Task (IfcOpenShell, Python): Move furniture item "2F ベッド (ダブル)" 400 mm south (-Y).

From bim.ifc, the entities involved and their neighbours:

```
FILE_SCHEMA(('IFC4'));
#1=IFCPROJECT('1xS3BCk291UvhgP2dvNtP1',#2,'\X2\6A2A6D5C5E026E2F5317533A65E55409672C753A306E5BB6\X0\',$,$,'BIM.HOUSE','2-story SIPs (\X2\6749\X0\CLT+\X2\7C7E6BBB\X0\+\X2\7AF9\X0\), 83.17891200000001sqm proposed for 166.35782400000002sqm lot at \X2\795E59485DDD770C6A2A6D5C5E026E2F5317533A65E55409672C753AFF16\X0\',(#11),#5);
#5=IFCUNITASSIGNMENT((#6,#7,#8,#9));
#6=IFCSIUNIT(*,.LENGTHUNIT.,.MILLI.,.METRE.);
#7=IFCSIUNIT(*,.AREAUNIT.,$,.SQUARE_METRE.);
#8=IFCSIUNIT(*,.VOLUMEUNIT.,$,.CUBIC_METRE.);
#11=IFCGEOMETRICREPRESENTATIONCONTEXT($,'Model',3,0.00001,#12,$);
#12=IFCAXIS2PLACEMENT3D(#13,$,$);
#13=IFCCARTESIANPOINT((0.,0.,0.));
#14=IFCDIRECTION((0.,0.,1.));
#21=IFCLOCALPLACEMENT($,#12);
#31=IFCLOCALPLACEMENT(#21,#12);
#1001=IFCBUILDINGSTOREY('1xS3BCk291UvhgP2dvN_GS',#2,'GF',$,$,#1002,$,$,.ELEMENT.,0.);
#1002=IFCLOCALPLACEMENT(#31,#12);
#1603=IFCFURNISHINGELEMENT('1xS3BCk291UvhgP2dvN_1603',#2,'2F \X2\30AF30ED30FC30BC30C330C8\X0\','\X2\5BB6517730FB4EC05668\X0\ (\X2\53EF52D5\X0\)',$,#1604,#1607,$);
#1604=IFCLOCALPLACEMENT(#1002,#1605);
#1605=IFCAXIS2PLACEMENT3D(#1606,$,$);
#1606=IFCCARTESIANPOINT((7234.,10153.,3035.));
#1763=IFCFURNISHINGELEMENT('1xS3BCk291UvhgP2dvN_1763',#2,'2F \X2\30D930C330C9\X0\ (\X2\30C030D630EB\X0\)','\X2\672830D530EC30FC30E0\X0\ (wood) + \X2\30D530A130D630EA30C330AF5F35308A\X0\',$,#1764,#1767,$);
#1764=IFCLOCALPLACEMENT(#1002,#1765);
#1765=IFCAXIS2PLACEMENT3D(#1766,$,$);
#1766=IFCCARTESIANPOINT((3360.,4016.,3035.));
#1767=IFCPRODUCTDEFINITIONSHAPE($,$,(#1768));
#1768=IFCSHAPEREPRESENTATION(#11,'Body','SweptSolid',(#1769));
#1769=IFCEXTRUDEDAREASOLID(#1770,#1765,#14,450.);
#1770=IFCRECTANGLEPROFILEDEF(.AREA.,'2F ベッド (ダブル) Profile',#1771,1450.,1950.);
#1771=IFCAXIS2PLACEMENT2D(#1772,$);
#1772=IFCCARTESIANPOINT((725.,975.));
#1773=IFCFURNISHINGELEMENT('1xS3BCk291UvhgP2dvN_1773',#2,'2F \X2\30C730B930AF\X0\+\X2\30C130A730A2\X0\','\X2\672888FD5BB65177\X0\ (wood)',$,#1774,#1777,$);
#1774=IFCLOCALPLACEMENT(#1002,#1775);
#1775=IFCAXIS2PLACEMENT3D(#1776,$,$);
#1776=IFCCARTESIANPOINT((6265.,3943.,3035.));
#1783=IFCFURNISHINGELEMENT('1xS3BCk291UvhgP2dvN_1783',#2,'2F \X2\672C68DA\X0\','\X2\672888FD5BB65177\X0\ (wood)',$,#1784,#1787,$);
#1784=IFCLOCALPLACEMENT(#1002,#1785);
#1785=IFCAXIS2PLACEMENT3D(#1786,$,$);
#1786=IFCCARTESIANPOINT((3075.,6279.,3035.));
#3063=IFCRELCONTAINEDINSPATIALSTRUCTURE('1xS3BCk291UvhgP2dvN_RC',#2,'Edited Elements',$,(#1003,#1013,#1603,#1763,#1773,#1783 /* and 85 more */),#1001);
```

```python
import ifcopenshell
import ifcopenshell.api.geometry
import ifcopenshell.util.placement
import ifcopenshell.util.unit

model = ifcopenshell.open("bim.ifc")
unit_scale = ifcopenshell.util.unit.calculate_unit_scale(model)

item = model.by_guid("1xS3BCk291UvhgP2dvN_1763")
matrix = ifcopenshell.util.placement.get_local_placement(item.ObjectPlacement)
matrix[1, 3] -= 0.4 / unit_scale
ifcopenshell.api.geometry.edit_object_placement(model, product=item, matrix=matrix, is_si=False)

print(ifcopenshell.util.placement.get_local_placement(item.ObjectPlacement).round(3) + 0.0)

model.write("bim_edited.ifc")
```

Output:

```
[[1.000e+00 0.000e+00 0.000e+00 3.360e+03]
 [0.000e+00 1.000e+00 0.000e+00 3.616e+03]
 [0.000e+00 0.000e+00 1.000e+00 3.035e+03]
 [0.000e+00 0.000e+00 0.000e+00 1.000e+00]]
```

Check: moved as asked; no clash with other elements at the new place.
